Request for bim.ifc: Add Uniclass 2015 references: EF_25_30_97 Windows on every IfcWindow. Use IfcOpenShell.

First a look at what the model holds.

```python
import ifcopenshell

model = ifcopenshell.open("bim.ifc")
print(model.schema)
print("classifications:", [c.Name for c in model.by_type("IfcClassification")])
for ifc_class in ("IfcDoor", "IfcRoof", "IfcStair", "IfcWall", "IfcWindow"):
    print(ifc_class, len(model.by_type(ifc_class)))
```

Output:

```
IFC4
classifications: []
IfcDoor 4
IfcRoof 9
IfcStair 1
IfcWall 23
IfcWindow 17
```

```python
import ifcopenshell
import ifcopenshell.api.classification

model = ifcopenshell.open("bim.ifc")

system = ifcopenshell.api.classification.add_classification(model, classification="Uniclass 2015")

codes = {
    "IfcWindow": ("EF_25_30_97", "Windows"),
}
for ifc_class, (code, name) in codes.items():
    products = model.by_type(ifc_class)
    ifcopenshell.api.classification.add_reference(
        model, products=products, classification=system, identification=code, name=name
    )
    print(code, len(products))

model.write("bim_edited.ifc")
```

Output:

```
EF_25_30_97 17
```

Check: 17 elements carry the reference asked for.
